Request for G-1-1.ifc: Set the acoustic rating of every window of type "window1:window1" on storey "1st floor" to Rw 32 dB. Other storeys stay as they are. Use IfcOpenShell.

First a look at what the model holds.

```python
import ifcopenshell
import ifcopenshell.util.element

model = ifcopenshell.open("G-1-1.ifc")
print(model.schema)
storey = next(s for s in model.by_type("IfcBuildingStorey") if s.Name == "1st floor")
windows = [e for e in ifcopenshell.util.element.get_decomposition(storey) if e.is_a("IfcWindow")]
seen = {}
for e in windows:
    element_type = ifcopenshell.util.element.get_type(e)
    key = (element_type.Name if element_type != e and element_type else None, ifcopenshell.util.element.get_pset(e, "Pset_WindowCommon", "AcousticRating"))
    seen[key] = seen.get(key, 0) + 1
for (name, value), count in sorted(seen.items(), key=str):
    print(count, "x", name, "|", value)
```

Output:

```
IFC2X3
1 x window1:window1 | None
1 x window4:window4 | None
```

```python
import ifcopenshell
import ifcopenshell.api.pset
import ifcopenshell.util.element

model = ifcopenshell.open("G-1-1.ifc")

storey = next(s for s in model.by_type("IfcBuildingStorey") if s.Name == "1st floor")
windows = [e for e in ifcopenshell.util.element.get_decomposition(storey) if e.is_a("IfcWindow")]

count = 0
for e in windows:
    element_type = ifcopenshell.util.element.get_type(e)
    if element_type in (None, e) or element_type.Name != "window1:window1":
        continue
    # add_pset returns the element's existing set when there is one.
    pset = ifcopenshell.api.pset.add_pset(model, product=e, name="Pset_WindowCommon")
    ifcopenshell.api.pset.edit_pset(model, pset=pset, properties={"AcousticRating": "Rw 32 dB"})
    count += 1

print(count, "windows updated")

model.write("G-1-1_edited.ifc")
```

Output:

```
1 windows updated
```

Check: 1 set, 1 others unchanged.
